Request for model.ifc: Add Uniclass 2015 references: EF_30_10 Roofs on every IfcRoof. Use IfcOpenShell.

First a look at what the model holds.

```python
import ifcopenshell

model = ifcopenshell.open("model.ifc")
print(model.schema)
print("classifications:", [c.Name for c in model.by_type("IfcClassification")])
for ifc_class in ("IfcDoor", "IfcRoof", "IfcStair", "IfcWall", "IfcWindow"):
    print(ifc_class, len(model.by_type(ifc_class)))
```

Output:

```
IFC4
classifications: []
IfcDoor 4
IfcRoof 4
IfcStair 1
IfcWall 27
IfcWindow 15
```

```python
import ifcopenshell
import ifcopenshell.api.classification

model = ifcopenshell.open("model.ifc")

system = ifcopenshell.api.classification.add_classification(model, classification="Uniclass 2015")

codes = {
    "IfcRoof": ("EF_30_10", "Roofs"),
}
for ifc_class, (code, name) in codes.items():
    products = model.by_type(ifc_class)
    ifcopenshell.api.classification.add_reference(
        model, products=products, classification=system, identification=code, name=name
    )
    print(code, len(products))

model.write("model_rev.ifc")
```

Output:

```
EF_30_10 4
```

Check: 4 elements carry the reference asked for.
